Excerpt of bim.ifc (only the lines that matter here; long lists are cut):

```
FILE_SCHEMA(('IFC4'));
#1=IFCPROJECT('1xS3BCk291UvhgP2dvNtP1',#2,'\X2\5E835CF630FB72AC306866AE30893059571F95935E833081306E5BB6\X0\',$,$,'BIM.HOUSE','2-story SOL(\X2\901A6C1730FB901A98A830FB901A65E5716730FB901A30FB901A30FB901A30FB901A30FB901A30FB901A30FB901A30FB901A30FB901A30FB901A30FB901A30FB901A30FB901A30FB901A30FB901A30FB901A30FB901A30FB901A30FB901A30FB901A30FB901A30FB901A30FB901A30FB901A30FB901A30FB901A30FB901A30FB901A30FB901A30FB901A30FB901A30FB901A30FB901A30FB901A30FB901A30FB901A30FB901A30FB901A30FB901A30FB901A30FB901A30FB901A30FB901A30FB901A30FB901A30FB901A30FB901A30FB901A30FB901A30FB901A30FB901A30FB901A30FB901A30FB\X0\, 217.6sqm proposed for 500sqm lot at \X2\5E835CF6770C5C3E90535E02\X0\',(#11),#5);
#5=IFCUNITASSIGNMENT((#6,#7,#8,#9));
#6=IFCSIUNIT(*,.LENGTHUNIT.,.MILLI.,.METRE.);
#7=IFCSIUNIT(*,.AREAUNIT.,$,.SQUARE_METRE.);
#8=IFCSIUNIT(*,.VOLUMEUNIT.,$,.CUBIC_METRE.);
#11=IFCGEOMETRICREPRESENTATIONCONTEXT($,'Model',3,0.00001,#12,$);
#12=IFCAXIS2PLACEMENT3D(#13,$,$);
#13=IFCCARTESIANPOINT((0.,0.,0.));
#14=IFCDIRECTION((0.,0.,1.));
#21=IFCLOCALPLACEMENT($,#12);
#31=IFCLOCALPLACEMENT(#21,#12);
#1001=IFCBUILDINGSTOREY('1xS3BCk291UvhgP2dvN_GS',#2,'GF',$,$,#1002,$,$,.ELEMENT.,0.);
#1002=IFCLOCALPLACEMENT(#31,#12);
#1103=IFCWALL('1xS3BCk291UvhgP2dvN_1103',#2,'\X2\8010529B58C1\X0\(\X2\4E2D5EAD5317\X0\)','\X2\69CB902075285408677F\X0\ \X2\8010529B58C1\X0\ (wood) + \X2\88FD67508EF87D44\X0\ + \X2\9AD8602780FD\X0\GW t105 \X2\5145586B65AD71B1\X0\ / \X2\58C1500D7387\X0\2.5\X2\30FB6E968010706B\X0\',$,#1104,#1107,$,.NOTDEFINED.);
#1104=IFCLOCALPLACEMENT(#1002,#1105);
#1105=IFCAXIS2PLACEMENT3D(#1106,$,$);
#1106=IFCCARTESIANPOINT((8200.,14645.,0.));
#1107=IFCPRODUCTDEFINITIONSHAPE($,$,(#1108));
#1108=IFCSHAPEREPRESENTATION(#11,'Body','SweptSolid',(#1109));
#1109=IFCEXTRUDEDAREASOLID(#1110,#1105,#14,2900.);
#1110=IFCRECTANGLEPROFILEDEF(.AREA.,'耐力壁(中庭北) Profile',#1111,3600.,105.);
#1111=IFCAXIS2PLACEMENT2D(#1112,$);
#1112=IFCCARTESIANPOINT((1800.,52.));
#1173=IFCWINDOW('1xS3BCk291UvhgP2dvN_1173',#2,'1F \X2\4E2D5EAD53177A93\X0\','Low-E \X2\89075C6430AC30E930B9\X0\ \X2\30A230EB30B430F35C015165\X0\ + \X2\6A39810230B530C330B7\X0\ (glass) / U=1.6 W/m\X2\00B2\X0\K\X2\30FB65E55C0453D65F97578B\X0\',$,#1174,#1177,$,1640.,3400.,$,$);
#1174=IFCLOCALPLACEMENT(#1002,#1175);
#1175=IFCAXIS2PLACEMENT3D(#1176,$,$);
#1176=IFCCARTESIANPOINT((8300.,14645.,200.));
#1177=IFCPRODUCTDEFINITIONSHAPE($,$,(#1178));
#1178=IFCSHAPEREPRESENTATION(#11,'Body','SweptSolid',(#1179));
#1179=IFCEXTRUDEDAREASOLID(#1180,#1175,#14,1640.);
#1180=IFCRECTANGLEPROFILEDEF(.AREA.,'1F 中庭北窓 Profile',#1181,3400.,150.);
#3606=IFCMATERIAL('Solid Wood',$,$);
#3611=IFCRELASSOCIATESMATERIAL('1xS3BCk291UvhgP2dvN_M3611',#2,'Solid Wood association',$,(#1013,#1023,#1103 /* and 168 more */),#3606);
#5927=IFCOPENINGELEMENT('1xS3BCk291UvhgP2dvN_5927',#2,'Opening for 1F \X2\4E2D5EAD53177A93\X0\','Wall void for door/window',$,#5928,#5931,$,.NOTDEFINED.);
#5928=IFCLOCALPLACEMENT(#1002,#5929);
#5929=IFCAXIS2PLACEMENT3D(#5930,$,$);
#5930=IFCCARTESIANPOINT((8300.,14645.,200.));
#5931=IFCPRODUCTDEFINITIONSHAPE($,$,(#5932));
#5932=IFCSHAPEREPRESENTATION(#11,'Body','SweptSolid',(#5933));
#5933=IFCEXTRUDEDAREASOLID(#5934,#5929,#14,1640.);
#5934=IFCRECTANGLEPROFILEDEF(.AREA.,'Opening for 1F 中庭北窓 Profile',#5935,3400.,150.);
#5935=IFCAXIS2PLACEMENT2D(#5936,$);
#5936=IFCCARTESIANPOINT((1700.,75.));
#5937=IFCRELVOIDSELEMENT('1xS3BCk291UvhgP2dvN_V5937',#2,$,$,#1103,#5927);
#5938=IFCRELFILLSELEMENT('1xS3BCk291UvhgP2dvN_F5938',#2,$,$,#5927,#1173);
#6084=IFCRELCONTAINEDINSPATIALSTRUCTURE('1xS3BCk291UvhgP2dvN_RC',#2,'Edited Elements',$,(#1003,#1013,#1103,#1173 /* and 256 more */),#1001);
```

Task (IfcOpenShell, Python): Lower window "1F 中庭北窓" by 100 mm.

```python
import numpy as np
import ifcopenshell
import ifcopenshell.api.geometry
import ifcopenshell.util.placement
import ifcopenshell.util.unit

model = ifcopenshell.open("bim.ifc")
unit_scale = ifcopenshell.util.unit.calculate_unit_scale(model)

window = model.by_guid("1xS3BCk291UvhgP2dvN_1173")
opening = window.FillsVoids[0].RelatingOpeningElement
dz = -0.1 / unit_scale

shift = np.array([0.0, 0.0, dz])
# The window is not placed relative to its opening, so move both.
for product in (opening, window):
    matrix = ifcopenshell.util.placement.get_local_placement(product.ObjectPlacement)
    matrix[:3, 3] += shift
    ifcopenshell.api.geometry.edit_object_placement(model, product=product, matrix=matrix, is_si=False)

print(f"moved by {dz * unit_scale:+.3f} m")

model.write("bim_updated.ifc")
```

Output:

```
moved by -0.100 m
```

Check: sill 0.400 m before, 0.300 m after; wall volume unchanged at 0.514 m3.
